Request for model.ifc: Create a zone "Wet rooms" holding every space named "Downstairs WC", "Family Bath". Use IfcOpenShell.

First a look at what the model holds.

```python
import ifcopenshell

model = ifcopenshell.open("model.ifc")
print(model.schema)
seen = {}
for space in model.by_type("IfcSpace"):
    seen[space.LongName] = seen.get(space.LongName, 0) + 1
for name, count in sorted(seen.items(), key=str):
    print(count, "x", name)
print("zones:", [z.Name for z in model.by_type("IfcZone")][:20])
```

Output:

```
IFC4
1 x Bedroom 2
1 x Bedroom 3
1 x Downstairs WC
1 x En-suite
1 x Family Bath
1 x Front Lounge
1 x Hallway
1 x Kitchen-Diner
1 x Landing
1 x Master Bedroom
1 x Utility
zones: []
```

```python
import ifcopenshell
import ifcopenshell.api.group
import ifcopenshell.api.root

model = ifcopenshell.open("model.ifc")

names = {"Downstairs WC", "Family Bath"}
spaces = [s for s in model.by_type("IfcSpace") if s.LongName in names]

zone = ifcopenshell.api.root.create_entity(model, ifc_class="IfcZone", name="Wet rooms")
ifcopenshell.api.group.assign_group(model, products=spaces, group=zone)
print(len(spaces), "spaces in", zone.Name)

model.write("model_v2.ifc")
```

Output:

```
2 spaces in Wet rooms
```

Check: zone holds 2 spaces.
